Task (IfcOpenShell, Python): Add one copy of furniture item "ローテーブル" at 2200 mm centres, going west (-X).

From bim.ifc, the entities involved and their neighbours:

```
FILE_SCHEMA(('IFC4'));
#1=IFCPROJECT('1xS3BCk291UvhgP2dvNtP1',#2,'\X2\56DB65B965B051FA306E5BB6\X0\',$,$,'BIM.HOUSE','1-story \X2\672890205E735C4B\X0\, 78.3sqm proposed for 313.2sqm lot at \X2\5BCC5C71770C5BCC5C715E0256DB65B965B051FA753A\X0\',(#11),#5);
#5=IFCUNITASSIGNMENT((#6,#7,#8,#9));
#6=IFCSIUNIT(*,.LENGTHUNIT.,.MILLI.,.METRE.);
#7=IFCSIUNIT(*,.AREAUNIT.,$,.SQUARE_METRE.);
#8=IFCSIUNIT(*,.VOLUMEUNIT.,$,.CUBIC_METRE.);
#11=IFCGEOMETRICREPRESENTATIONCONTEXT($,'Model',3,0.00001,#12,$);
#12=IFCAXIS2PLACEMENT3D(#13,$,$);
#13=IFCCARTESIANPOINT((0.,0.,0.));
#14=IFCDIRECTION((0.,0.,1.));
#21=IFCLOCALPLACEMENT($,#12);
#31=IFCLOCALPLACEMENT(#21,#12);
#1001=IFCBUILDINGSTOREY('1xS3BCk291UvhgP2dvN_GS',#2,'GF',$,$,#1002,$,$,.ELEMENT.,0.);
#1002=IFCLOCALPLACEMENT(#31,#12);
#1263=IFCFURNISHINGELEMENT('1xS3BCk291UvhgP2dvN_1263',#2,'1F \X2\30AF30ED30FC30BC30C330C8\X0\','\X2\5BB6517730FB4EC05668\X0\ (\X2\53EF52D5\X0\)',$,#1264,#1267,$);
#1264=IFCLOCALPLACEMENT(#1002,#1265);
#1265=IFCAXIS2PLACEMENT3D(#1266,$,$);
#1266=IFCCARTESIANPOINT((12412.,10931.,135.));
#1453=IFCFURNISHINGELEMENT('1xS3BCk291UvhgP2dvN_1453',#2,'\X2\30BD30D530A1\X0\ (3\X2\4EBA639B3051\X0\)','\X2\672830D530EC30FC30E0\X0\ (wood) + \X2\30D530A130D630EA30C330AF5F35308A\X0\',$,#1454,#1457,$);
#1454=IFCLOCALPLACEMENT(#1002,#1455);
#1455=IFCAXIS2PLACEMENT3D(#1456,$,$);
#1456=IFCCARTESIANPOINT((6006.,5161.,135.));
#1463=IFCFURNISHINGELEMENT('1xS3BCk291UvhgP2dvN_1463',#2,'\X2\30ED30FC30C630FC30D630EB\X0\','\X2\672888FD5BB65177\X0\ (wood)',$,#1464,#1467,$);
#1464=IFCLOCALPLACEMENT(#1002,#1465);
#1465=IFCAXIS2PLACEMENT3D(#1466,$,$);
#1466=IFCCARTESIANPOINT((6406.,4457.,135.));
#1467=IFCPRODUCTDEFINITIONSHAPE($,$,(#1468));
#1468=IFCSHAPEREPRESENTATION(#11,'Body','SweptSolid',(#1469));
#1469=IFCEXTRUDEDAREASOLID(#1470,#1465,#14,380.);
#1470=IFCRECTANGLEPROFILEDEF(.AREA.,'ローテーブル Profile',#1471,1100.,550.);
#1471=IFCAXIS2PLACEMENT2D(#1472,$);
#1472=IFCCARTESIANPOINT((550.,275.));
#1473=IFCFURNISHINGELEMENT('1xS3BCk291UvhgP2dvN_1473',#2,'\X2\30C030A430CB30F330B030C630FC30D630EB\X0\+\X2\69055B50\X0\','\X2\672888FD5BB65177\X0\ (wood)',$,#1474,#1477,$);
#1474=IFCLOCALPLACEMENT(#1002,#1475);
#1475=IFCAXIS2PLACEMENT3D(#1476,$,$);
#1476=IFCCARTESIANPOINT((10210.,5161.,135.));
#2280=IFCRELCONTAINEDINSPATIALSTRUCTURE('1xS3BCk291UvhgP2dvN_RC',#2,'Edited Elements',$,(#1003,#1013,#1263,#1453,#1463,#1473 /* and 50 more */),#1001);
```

```python
import numpy as np
import ifcopenshell
import ifcopenshell.api.geometry
import ifcopenshell.api.root
import ifcopenshell.util.element
import ifcopenshell.util.placement
import ifcopenshell.util.unit

model = ifcopenshell.open("bim.ifc")
unit_scale = ifcopenshell.util.unit.calculate_unit_scale(model)


def reuse_history(source, copy):
    """copy_class also copies each property set's owner history, people and application; keep the originals."""
    for rel in copy.IsDefinedBy:
        if rel.is_a("IfcRelDefinesByProperties") and (history := rel.RelatingPropertyDefinition.OwnerHistory):
            rel.RelatingPropertyDefinition.OwnerHistory = source.OwnerHistory
            ifcopenshell.util.element.remove_deep2(model, history)


source = model.by_guid("1xS3BCk291UvhgP2dvN_1463")
base = ifcopenshell.util.placement.get_local_placement(source.ObjectPlacement)
step = np.array([-1.0, 0.0, 0.0]) * 2.2 / unit_scale

for i in range(1, 2):
    copy = ifcopenshell.api.root.copy_class(model, product=source)
    copy.Representation = ifcopenshell.util.element.copy_deep(
        model, source.Representation, exclude=["IfcGeometricRepresentationContext", "IfcRepresentationMap"]
    )
    reuse_history(source, copy)
    matrix = base.copy()
    matrix[:3, 3] += i * step
    print("added at", matrix[:3, 3].round(3) + 0.0)
    ifcopenshell.api.geometry.edit_object_placement(model, product=copy, matrix=matrix, is_si=False)

model.write("bim_rev.ifc")
```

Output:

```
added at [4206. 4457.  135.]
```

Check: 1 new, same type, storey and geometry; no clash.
